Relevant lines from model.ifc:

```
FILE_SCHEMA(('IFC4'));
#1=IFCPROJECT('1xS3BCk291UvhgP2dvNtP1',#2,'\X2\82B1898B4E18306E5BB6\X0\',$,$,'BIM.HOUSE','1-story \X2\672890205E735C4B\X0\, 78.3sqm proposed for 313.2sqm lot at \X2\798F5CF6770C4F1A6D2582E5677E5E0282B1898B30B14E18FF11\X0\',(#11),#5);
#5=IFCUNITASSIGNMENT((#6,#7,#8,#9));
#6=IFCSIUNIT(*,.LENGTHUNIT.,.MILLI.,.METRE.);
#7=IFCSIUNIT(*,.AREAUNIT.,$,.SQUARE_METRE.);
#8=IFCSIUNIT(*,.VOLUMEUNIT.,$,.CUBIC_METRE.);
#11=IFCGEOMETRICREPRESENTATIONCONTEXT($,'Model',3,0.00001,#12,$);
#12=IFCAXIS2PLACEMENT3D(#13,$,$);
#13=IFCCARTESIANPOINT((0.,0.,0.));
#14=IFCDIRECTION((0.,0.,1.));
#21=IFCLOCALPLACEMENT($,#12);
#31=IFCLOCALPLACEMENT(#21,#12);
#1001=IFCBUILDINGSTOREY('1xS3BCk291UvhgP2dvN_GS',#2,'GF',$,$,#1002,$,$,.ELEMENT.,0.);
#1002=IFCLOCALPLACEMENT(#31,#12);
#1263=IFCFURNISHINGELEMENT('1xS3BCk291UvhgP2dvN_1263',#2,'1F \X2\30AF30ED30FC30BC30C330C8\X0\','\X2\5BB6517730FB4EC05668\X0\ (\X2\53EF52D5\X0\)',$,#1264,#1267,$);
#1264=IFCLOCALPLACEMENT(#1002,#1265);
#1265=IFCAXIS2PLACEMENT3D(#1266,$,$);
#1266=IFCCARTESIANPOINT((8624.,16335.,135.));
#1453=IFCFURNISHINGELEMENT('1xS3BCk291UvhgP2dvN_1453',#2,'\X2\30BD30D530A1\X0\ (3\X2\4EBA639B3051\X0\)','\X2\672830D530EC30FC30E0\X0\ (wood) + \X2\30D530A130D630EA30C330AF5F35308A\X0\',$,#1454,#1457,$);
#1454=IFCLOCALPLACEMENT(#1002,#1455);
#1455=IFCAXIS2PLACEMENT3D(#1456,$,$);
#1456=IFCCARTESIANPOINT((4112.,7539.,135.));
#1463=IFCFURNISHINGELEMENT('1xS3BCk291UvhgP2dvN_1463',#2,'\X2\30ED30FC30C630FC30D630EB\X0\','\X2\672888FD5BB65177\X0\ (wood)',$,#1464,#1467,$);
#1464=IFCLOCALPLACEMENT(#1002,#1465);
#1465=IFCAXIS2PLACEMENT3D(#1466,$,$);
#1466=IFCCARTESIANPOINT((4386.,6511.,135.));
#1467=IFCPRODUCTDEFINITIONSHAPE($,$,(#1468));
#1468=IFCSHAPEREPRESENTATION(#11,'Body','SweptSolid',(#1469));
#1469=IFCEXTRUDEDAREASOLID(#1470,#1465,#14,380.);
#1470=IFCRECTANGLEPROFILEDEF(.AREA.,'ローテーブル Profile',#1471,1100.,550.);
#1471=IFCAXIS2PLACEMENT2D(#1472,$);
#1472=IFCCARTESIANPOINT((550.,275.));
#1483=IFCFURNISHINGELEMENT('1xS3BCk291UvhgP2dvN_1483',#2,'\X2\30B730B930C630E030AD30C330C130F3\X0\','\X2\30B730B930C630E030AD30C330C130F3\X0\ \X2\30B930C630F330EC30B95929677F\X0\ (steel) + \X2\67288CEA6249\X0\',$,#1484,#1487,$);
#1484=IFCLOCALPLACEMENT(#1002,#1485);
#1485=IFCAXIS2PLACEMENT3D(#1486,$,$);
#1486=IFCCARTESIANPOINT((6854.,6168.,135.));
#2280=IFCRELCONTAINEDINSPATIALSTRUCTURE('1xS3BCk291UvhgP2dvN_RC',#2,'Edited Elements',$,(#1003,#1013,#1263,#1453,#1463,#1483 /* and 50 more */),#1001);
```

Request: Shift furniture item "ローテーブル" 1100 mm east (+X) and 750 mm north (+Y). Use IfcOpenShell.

```python
import ifcopenshell
import ifcopenshell.api.geometry
import ifcopenshell.util.placement
import ifcopenshell.util.unit

model = ifcopenshell.open("model.ifc")
unit_scale = ifcopenshell.util.unit.calculate_unit_scale(model)

item = model.by_guid("1xS3BCk291UvhgP2dvN_1463")
matrix = ifcopenshell.util.placement.get_local_placement(item.ObjectPlacement)
matrix[0, 3] += 1.1 / unit_scale
matrix[1, 3] += 0.75 / unit_scale
ifcopenshell.api.geometry.edit_object_placement(model, product=item, matrix=matrix, is_si=False)

print(ifcopenshell.util.placement.get_local_placement(item.ObjectPlacement).round(3) + 0.0)

model.write("model-out.ifc")
```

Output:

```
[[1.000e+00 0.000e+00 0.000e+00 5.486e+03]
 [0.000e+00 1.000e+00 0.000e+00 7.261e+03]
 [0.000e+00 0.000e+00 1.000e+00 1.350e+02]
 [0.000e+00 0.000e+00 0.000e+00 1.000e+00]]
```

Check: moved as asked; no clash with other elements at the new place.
